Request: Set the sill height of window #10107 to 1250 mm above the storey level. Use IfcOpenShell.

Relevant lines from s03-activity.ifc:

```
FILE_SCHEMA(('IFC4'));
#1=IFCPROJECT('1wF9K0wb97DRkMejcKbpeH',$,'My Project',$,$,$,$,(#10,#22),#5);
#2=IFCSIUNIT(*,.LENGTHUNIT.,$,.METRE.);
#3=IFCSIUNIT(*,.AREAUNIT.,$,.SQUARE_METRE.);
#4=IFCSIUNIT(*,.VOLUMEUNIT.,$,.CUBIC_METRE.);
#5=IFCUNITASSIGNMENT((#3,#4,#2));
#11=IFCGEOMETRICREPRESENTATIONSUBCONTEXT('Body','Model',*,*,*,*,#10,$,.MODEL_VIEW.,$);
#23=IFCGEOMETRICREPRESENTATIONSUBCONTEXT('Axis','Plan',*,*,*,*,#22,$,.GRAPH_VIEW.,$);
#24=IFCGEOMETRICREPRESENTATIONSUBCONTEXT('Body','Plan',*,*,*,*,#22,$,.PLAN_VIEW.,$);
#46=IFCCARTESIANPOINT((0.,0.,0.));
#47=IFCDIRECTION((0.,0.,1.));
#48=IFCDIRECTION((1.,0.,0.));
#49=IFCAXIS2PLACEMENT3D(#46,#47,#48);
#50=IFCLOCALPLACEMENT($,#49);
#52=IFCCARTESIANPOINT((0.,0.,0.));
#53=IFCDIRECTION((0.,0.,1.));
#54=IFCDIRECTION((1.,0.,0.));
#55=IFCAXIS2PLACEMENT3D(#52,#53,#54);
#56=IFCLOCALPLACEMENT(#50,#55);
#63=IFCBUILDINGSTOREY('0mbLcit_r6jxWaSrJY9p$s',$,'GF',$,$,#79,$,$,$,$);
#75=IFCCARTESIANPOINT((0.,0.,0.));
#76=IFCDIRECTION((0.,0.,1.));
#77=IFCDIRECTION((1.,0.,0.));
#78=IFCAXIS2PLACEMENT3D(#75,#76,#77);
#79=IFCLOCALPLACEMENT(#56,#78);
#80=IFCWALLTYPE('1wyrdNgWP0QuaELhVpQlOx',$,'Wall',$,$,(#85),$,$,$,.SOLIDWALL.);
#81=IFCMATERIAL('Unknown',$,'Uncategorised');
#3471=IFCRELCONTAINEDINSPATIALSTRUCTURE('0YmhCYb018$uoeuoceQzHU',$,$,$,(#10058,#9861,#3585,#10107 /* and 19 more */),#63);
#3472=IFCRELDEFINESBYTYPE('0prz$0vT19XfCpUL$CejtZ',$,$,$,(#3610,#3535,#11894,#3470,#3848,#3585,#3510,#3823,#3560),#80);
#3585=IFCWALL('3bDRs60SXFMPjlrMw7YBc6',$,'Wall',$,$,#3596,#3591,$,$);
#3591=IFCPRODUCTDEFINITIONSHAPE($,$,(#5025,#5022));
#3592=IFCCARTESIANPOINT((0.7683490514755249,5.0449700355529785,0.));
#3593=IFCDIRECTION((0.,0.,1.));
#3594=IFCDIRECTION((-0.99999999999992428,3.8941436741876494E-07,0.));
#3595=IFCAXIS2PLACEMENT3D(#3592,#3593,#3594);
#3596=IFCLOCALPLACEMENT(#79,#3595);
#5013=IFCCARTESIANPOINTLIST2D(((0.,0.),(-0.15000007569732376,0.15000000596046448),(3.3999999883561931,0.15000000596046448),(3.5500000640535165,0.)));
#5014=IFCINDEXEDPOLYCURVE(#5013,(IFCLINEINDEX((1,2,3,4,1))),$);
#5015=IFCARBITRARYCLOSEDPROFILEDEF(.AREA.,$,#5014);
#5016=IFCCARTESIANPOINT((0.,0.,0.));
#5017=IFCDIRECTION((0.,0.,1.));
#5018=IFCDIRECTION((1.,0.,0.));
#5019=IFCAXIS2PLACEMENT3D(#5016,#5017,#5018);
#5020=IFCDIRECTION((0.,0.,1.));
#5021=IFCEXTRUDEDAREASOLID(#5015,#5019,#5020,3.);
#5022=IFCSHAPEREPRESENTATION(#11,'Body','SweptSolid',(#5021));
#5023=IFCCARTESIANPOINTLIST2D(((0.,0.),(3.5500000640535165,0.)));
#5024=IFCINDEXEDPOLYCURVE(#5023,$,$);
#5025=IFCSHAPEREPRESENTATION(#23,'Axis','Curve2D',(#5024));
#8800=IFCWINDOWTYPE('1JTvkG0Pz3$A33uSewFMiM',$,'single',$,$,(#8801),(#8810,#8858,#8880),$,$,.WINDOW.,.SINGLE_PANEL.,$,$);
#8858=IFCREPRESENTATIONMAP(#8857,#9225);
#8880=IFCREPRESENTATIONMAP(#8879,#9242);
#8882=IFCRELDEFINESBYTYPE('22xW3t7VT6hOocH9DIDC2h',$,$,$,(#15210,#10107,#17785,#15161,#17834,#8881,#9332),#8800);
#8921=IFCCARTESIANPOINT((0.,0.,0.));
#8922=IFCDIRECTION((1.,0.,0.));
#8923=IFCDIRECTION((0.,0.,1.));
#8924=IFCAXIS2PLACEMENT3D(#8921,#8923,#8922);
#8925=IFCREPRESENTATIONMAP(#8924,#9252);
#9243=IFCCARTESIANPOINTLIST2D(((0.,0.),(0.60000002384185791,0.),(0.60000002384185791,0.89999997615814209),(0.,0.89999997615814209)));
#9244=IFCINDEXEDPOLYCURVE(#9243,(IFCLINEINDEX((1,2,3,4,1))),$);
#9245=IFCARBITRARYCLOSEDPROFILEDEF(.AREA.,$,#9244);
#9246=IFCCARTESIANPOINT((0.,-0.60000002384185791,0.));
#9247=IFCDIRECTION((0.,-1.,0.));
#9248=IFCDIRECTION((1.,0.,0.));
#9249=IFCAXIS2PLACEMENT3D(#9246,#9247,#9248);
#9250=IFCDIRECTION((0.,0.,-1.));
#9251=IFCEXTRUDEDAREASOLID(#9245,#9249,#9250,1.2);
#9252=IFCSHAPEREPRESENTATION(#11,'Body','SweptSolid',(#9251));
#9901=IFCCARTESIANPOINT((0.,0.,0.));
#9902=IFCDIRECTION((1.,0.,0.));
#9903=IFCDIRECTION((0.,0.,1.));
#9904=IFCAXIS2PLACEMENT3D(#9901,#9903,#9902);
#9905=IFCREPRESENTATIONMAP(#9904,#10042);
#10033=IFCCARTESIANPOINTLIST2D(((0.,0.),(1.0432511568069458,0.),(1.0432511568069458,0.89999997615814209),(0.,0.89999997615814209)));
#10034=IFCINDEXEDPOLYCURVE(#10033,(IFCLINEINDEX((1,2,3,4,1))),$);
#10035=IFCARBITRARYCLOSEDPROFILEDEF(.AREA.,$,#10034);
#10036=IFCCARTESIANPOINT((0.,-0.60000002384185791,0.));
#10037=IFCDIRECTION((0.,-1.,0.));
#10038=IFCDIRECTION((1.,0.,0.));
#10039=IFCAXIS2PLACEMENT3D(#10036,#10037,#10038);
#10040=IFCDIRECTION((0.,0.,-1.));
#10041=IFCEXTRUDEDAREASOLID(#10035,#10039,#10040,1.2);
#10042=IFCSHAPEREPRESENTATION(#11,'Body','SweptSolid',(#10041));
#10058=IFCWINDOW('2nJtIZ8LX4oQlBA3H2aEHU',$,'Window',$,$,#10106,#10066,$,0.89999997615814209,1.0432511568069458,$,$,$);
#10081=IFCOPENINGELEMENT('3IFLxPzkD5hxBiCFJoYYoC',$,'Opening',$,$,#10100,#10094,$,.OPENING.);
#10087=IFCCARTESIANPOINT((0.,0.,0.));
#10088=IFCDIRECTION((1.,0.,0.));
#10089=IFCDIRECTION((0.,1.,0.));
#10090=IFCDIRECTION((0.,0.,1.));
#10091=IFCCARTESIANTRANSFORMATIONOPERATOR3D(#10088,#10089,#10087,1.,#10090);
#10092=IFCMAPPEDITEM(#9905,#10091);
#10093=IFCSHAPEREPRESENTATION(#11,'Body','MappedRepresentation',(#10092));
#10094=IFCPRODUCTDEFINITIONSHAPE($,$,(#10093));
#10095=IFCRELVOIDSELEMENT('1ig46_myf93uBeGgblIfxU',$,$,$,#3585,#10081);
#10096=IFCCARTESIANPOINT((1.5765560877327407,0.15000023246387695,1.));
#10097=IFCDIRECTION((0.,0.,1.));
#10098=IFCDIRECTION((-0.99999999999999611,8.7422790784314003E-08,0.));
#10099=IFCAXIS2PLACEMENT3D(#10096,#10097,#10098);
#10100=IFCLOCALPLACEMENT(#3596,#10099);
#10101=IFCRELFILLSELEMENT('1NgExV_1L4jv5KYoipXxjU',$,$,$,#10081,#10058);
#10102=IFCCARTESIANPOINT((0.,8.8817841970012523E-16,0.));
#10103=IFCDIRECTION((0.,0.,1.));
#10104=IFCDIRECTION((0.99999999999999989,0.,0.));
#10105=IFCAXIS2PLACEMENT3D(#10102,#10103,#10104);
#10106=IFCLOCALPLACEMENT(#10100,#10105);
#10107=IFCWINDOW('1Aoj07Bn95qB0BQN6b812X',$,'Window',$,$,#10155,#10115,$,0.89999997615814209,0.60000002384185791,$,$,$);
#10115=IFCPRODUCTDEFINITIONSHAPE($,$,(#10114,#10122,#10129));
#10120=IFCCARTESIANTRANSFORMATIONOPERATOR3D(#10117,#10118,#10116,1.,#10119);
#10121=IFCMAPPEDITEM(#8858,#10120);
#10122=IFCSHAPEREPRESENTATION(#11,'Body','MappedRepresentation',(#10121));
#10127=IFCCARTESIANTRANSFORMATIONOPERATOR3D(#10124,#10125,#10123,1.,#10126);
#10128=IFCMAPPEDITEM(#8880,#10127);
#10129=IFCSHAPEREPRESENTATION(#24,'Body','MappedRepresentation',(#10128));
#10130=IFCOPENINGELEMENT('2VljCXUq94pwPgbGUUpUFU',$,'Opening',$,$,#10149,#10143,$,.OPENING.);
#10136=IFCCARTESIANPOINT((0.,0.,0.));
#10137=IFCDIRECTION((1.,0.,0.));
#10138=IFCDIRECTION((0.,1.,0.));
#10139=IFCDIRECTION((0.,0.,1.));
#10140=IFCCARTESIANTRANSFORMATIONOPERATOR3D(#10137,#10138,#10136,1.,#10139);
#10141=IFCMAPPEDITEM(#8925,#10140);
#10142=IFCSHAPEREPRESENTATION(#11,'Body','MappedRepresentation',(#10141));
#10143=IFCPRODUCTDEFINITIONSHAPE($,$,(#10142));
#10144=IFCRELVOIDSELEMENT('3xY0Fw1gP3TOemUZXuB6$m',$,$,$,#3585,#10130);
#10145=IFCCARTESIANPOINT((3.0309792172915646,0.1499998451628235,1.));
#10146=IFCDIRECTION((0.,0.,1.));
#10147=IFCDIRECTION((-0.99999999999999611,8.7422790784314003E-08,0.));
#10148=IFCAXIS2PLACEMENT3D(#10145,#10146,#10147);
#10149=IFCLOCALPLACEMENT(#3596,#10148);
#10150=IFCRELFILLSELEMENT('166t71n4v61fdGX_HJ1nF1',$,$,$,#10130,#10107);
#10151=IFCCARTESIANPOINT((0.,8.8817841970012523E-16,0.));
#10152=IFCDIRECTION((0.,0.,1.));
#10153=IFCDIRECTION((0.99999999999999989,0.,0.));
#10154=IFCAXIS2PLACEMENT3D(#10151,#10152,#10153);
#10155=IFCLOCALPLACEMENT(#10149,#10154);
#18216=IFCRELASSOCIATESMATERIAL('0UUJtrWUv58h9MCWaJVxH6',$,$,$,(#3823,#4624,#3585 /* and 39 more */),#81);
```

```python
import numpy as np
import ifcopenshell
import ifcopenshell.api.geometry
import ifcopenshell.geom
import ifcopenshell.util.element
import ifcopenshell.util.placement
import ifcopenshell.util.shape
import ifcopenshell.util.unit

model = ifcopenshell.open("s03-activity.ifc")
unit_scale = ifcopenshell.util.unit.calculate_unit_scale(model)

window = model.by_id(10107)
opening = window.FillsVoids[0].RelatingOpeningElement
storey = ifcopenshell.util.element.get_container(window, ifc_class="IfcBuildingStorey")
level = ifcopenshell.util.placement.get_local_placement(storey.ObjectPlacement)[2, 3]

# The opening's origin need not be at the sill, so measure its lowest point.
shape = ifcopenshell.geom.create_shape(ifcopenshell.geom.settings(), opening)
bottom = ifcopenshell.util.shape.get_shape_bottom_elevation(shape, shape.geometry) / unit_scale
dz = level + 1.25 / unit_scale - bottom

shift = np.array([0.0, 0.0, dz])
# The window is placed relative to its opening, so it follows when the opening moves.
matrix = ifcopenshell.util.placement.get_local_placement(opening.ObjectPlacement)
matrix[:3, 3] += shift
ifcopenshell.api.geometry.edit_object_placement(
    model, product=opening, matrix=matrix, is_si=False, should_transform_children=True
)

print(f"moved by {dz * unit_scale:+.3f} m")

model.write("s03-activity-out.ifc")
```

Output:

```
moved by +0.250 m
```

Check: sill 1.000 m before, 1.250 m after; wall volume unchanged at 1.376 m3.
